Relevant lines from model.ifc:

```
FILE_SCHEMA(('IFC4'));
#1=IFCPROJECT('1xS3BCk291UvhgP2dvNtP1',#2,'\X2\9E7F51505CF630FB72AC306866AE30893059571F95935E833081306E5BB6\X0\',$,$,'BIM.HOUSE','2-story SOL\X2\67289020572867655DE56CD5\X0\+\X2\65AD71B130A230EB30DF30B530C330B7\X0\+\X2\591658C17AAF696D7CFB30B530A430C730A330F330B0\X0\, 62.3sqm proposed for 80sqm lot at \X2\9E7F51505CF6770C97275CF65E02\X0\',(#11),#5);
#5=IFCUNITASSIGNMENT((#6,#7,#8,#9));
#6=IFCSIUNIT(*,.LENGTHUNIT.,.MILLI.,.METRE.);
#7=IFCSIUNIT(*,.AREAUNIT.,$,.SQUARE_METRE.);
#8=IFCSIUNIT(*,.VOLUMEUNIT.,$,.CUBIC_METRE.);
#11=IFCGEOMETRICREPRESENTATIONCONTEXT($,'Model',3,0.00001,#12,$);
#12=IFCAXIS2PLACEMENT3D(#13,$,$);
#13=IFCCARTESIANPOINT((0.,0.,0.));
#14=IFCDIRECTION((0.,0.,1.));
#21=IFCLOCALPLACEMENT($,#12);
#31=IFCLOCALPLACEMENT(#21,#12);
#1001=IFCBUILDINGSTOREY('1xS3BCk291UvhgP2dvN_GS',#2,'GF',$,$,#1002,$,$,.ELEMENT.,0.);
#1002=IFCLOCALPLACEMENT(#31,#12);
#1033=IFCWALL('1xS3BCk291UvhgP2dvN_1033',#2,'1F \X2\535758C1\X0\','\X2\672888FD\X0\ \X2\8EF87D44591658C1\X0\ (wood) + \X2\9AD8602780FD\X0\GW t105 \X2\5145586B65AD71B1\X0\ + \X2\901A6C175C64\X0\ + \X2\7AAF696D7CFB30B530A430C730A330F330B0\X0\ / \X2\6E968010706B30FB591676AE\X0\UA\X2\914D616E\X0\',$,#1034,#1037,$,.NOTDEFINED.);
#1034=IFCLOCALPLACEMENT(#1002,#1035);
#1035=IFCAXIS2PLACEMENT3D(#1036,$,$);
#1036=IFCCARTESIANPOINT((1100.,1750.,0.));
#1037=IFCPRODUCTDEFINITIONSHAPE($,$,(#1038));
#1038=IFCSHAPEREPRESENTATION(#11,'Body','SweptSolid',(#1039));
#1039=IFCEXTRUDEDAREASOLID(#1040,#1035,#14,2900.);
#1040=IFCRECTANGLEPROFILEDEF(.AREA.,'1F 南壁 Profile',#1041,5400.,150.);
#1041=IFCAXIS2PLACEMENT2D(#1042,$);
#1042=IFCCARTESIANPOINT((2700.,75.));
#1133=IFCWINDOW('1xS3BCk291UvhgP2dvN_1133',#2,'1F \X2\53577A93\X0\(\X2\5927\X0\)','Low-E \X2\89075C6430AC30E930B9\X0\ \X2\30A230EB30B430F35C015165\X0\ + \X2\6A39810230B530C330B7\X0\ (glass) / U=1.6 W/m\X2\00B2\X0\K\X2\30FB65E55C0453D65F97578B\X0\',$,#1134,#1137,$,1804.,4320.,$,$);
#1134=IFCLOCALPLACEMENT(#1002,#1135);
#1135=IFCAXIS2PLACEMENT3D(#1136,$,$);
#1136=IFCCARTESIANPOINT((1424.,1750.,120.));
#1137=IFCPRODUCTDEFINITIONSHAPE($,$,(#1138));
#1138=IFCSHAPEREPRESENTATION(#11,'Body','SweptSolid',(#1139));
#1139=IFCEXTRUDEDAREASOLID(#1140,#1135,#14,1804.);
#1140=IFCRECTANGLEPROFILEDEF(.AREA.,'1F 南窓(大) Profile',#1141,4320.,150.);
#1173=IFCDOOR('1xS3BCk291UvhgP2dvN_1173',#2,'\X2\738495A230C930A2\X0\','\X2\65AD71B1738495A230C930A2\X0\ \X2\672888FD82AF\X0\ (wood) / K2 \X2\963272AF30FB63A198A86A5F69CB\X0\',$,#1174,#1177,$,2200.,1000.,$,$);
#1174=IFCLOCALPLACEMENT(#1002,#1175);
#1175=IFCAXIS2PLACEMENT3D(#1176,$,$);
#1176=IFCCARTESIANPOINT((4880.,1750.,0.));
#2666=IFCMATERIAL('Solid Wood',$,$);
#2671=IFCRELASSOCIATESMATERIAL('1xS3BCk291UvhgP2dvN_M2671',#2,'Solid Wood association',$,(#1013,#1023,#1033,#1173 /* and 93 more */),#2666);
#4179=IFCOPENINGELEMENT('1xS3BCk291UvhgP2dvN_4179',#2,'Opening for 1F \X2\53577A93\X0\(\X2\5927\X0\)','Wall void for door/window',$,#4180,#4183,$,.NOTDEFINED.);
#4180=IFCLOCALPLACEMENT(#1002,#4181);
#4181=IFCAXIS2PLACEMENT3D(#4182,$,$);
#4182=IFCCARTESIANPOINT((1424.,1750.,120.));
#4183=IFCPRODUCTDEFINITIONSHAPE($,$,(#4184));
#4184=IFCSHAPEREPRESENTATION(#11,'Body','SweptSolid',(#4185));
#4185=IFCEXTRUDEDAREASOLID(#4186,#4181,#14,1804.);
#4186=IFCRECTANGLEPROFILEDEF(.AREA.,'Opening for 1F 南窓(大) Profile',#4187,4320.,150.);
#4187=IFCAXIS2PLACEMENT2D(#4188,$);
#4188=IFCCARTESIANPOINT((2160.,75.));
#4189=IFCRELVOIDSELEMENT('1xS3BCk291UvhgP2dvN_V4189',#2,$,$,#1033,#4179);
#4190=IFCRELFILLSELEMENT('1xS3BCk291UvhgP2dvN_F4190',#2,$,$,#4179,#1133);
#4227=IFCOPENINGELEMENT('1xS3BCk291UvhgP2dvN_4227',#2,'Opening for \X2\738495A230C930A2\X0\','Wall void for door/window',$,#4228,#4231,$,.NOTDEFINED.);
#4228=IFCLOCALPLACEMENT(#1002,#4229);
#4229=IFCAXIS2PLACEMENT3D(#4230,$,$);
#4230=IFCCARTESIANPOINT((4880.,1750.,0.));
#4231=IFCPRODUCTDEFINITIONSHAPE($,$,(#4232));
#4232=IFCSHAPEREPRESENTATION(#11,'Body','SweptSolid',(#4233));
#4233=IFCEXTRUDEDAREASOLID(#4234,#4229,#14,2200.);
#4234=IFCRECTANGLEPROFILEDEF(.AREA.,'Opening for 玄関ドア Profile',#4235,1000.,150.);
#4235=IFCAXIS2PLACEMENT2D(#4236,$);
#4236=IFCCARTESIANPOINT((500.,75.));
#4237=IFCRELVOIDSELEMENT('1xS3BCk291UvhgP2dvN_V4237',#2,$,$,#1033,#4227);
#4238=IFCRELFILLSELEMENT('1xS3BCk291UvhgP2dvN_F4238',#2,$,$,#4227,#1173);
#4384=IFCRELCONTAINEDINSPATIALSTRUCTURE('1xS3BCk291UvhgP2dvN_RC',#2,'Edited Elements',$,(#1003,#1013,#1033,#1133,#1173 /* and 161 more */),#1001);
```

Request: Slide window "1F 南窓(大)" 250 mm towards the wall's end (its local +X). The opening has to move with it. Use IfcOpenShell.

```python
import ifcopenshell
import ifcopenshell.api.geometry
import ifcopenshell.util.placement

model = ifcopenshell.open("model.ifc")

window = model.by_guid("1xS3BCk291UvhgP2dvN_1133")
opening = window.FillsVoids[0].RelatingOpeningElement
wall = opening.VoidsElements[0].RelatingBuildingElement

wall_matrix = ifcopenshell.util.placement.get_local_placement(wall.ObjectPlacement)
shift = wall_matrix[:3, 0] * 250.0
before = ifcopenshell.util.placement.get_local_placement(window.ObjectPlacement)[:3, 3].copy()

# The window is not placed relative to its opening, so move both.
for product in (opening, window):
    matrix = ifcopenshell.util.placement.get_local_placement(product.ObjectPlacement)
    matrix[:3, 3] += shift
    ifcopenshell.api.geometry.edit_object_placement(model, product=product, matrix=matrix, is_si=False)

after = ifcopenshell.util.placement.get_local_placement(window.ObjectPlacement)[:3, 3]
print("window moved by", (after - before).round(3) + 0.0)

model.write("model_updated.ifc")
```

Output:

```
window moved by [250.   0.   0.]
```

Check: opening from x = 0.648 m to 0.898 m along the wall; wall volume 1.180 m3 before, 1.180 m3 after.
